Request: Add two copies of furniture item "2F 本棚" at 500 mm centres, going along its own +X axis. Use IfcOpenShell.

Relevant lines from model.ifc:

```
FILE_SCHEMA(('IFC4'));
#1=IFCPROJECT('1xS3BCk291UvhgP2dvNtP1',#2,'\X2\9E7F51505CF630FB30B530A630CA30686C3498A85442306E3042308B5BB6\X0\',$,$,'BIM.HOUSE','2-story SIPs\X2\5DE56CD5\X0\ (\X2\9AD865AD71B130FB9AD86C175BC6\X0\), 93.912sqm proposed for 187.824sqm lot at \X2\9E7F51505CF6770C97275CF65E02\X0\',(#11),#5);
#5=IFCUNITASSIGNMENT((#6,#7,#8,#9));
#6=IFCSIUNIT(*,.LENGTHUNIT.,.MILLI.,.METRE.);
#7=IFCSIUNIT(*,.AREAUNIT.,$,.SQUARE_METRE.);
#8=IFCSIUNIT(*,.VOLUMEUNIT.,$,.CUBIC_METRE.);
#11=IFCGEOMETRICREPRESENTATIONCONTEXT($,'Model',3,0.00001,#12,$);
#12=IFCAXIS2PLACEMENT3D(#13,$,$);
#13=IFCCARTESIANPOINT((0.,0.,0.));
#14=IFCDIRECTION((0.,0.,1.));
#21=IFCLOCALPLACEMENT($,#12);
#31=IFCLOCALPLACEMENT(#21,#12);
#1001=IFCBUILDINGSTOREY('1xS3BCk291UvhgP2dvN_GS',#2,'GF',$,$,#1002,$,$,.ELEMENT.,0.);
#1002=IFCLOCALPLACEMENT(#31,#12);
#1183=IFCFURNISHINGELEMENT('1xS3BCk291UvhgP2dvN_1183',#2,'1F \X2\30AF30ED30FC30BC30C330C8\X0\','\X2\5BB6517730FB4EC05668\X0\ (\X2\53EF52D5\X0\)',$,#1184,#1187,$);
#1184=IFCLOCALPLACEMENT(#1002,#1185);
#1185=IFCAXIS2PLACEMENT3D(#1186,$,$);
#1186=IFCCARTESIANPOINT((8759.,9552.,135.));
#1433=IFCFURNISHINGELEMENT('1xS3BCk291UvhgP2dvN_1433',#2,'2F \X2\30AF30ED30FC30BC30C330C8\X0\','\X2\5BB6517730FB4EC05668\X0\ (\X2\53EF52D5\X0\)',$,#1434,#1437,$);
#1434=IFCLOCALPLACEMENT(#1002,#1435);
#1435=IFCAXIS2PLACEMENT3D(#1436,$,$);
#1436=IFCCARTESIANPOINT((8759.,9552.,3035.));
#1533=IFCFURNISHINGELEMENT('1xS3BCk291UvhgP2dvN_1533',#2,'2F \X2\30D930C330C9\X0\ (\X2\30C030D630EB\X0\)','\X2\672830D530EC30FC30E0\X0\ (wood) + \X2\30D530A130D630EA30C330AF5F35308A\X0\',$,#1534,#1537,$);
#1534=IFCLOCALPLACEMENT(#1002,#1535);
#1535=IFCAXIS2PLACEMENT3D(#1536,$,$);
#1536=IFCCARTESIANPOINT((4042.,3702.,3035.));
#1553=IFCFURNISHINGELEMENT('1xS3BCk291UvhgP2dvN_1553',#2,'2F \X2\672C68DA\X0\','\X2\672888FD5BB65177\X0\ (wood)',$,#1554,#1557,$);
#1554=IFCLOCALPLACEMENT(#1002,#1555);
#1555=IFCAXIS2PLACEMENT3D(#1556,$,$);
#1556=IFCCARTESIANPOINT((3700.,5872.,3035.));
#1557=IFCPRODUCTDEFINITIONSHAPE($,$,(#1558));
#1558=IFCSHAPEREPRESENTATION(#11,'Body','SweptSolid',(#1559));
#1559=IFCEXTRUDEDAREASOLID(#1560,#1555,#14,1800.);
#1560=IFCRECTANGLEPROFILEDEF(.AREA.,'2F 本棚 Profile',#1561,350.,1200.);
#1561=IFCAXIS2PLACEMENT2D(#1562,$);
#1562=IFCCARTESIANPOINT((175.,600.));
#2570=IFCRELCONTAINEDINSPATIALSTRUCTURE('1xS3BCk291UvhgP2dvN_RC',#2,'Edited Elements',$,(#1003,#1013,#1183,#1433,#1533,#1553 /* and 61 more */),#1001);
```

```python
import ifcopenshell
import ifcopenshell.api.geometry
import ifcopenshell.api.root
import ifcopenshell.util.element
import ifcopenshell.util.placement
import ifcopenshell.util.unit

model = ifcopenshell.open("model.ifc")
unit_scale = ifcopenshell.util.unit.calculate_unit_scale(model)


def reuse_history(source, copy):
    """copy_class also copies each property set's owner history, people and application; keep the originals."""
    for rel in copy.IsDefinedBy:
        if rel.is_a("IfcRelDefinesByProperties") and (history := rel.RelatingPropertyDefinition.OwnerHistory):
            rel.RelatingPropertyDefinition.OwnerHistory = source.OwnerHistory
            ifcopenshell.util.element.remove_deep2(model, history)


source = model.by_guid("1xS3BCk291UvhgP2dvN_1553")
base = ifcopenshell.util.placement.get_local_placement(source.ObjectPlacement)
step = base[:3, 0] * 0.5 / unit_scale

for i in range(1, 3):
    copy = ifcopenshell.api.root.copy_class(model, product=source)
    copy.Representation = ifcopenshell.util.element.copy_deep(
        model, source.Representation, exclude=["IfcGeometricRepresentationContext", "IfcRepresentationMap"]
    )
    reuse_history(source, copy)
    matrix = base.copy()
    matrix[:3, 3] += i * step
    print("added at", matrix[:3, 3].round(3) + 0.0)
    ifcopenshell.api.geometry.edit_object_placement(model, product=copy, matrix=matrix, is_si=False)

model.write("model_rev.ifc")
```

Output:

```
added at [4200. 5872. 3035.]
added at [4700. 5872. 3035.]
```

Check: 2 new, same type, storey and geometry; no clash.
